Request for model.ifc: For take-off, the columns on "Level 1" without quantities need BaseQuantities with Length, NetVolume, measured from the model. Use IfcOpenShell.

First a look at what the model holds.

```python
import ifcopenshell
import ifcopenshell.util.element
import ifcopenshell.util.unit

model = ifcopenshell.open("model.ifc")
print(model.schema)
for unit_type in ("LENGTHUNIT", "AREAUNIT", "VOLUMEUNIT"):
    print(unit_type, ifcopenshell.util.unit.calculate_unit_scale(model, unit_type))
storey = next(s for s in model.by_type("IfcBuildingStorey") if s.Name == "Level 1")
columns = [e for e in ifcopenshell.util.element.get_decomposition(storey) if e.is_a("IfcColumn")]
for e in sorted(columns, key=lambda e: e.id()):
    print(e.id(), e.is_a(), e.Name, list(ifcopenshell.util.element.get_psets(e, qtos_only=True)), sep=" | ")
```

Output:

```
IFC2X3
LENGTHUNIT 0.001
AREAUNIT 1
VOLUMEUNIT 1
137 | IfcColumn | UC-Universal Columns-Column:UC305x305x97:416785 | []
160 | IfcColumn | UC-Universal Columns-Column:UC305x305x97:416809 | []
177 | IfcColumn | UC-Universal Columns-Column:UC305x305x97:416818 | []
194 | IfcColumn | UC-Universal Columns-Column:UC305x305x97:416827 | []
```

```python
import ifcopenshell
import ifcopenshell.api.pset
import ifcopenshell.geom
import ifcopenshell.util.element
import ifcopenshell.util.shape
import ifcopenshell.util.unit

model = ifcopenshell.open("model.ifc")
unit_scale = ifcopenshell.util.unit.calculate_unit_scale(model)
volume_scale = ifcopenshell.util.unit.calculate_unit_scale(model, "VOLUMEUNIT")
settings = ifcopenshell.geom.settings()

storey = next(s for s in model.by_type("IfcBuildingStorey") if s.Name == "Level 1")
columns = [e for e in ifcopenshell.util.element.get_decomposition(storey) if e.is_a("IfcColumn")]

for e in sorted(columns, key=lambda e: e.id()):
    if ifcopenshell.util.element.get_psets(e, qtos_only=True, should_inherit=False):
        continue
    # Geometry comes back in metres, in the element's own axes.
    shape = ifcopenshell.geom.create_shape(settings, e)
    values = {
        "Length": ifcopenshell.util.shape.get_z(shape.geometry) / unit_scale,
        "NetVolume": ifcopenshell.util.shape.get_volume(shape.geometry) / volume_scale,
    }
    qto = ifcopenshell.api.pset.add_qto(model, product=e, name="BaseQuantities")
    ifcopenshell.api.pset.edit_qto(model, qto=qto, properties=values)
    print(e.id(), {k: round(v, 3) for k, v in values.items()})

model.write("model-out.ifc")
```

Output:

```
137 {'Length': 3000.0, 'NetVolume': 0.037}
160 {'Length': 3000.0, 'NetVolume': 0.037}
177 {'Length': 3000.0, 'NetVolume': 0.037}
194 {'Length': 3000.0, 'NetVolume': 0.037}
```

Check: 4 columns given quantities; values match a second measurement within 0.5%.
